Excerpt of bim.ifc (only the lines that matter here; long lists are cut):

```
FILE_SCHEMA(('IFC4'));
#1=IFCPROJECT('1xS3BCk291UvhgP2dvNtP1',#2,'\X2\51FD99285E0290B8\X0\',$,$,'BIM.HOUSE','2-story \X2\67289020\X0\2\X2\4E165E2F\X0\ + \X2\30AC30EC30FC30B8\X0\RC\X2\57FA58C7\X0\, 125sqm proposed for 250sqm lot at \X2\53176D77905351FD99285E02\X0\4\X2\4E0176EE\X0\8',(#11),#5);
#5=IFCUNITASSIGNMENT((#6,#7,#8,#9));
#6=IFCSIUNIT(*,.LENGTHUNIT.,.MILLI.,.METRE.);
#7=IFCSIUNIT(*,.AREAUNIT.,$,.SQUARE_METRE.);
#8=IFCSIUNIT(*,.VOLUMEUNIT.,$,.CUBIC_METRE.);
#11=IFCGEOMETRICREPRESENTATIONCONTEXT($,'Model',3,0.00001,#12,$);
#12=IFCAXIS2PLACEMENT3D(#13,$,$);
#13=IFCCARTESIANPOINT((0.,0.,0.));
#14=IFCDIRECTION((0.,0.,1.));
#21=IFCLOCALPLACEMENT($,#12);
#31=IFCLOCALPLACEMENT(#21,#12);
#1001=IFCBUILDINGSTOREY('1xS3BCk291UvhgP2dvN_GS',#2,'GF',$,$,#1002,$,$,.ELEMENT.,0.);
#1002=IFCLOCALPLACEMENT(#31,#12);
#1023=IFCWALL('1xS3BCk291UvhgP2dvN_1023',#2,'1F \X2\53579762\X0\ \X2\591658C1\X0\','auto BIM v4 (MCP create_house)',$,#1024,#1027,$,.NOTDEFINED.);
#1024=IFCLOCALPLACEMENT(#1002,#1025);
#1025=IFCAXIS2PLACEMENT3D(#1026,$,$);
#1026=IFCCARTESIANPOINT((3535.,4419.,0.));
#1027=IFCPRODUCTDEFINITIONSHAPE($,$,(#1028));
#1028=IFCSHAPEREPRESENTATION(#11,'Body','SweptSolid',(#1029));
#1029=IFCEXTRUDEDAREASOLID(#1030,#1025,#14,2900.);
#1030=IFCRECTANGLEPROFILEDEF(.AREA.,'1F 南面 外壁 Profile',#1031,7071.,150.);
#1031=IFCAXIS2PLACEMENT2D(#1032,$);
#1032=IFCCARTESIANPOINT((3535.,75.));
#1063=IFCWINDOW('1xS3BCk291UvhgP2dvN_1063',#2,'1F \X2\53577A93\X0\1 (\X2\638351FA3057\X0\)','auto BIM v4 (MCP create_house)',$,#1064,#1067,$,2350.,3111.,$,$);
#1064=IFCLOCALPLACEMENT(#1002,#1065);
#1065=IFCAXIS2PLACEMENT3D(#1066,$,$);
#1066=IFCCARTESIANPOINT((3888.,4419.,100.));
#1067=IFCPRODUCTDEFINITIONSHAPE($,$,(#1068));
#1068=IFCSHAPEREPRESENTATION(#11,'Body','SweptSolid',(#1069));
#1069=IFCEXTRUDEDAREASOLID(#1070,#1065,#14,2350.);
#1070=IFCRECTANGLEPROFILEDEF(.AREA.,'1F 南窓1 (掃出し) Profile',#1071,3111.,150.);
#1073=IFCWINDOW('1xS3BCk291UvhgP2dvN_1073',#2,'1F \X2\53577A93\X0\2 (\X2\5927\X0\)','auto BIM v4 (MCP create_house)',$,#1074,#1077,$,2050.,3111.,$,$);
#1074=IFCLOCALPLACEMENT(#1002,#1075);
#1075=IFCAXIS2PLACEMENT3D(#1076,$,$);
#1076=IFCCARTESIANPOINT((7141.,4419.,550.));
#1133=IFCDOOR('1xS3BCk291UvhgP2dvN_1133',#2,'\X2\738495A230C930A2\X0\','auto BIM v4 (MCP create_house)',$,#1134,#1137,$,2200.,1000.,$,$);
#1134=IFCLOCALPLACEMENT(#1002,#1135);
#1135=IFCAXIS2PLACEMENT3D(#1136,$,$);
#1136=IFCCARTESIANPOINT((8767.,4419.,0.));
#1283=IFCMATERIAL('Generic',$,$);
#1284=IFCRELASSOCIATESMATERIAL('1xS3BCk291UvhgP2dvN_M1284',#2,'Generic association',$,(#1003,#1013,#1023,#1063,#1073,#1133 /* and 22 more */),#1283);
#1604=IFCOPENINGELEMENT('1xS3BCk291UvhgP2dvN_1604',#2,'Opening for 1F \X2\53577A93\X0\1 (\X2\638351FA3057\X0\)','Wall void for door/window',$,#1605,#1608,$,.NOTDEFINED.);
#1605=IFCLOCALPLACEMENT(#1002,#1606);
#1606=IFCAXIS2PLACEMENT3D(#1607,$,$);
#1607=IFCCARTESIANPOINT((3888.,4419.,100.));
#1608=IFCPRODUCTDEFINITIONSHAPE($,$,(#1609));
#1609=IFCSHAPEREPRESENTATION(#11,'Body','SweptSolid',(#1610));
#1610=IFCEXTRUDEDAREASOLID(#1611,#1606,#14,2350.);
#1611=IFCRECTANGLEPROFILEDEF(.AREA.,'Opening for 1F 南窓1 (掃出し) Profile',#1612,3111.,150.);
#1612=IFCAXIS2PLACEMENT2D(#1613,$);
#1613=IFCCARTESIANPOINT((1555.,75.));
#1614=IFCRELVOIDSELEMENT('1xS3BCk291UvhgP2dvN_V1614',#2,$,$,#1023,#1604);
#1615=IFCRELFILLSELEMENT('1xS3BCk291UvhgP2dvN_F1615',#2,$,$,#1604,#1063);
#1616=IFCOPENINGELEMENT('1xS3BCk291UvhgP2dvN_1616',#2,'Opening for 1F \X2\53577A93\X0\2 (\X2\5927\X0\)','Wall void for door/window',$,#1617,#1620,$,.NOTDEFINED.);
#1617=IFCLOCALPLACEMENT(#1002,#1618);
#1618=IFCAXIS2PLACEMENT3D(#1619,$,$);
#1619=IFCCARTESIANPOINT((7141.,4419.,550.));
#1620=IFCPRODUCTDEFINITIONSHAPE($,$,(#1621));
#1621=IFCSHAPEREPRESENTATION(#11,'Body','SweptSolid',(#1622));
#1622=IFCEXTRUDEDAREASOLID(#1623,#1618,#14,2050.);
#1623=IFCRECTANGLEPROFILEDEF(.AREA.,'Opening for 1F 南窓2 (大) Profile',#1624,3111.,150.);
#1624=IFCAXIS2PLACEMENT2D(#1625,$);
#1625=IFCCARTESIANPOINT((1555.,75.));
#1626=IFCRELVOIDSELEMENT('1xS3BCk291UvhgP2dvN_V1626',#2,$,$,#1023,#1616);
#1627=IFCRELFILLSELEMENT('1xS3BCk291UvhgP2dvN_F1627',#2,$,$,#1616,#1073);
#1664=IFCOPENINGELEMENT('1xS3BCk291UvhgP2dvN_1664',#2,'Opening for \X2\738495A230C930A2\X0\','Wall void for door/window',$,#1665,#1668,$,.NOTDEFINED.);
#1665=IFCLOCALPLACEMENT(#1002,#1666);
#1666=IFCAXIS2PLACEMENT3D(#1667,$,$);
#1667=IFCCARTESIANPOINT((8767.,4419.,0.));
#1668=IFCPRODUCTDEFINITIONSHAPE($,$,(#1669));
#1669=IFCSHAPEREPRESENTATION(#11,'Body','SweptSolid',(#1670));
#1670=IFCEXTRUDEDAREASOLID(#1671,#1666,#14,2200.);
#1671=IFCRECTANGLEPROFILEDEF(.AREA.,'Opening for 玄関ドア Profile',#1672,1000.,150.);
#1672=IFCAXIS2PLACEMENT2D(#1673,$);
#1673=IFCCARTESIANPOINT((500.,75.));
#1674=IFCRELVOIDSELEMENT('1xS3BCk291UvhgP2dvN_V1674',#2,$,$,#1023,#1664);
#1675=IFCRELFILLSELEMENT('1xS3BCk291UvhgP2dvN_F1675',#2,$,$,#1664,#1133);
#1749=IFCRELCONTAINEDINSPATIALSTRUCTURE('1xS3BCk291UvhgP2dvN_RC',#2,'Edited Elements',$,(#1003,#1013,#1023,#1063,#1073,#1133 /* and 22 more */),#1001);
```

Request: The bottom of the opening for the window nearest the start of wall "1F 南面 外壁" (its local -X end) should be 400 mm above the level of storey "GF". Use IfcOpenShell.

```python
import numpy as np
import ifcopenshell
import ifcopenshell.api.geometry
import ifcopenshell.geom
import ifcopenshell.util.element
import ifcopenshell.util.placement
import ifcopenshell.util.shape
import ifcopenshell.util.unit

model = ifcopenshell.open("bim.ifc")
unit_scale = ifcopenshell.util.unit.calculate_unit_scale(model)

window = model.by_guid("1xS3BCk291UvhgP2dvN_1063")
opening = window.FillsVoids[0].RelatingOpeningElement
storey = ifcopenshell.util.element.get_container(window, ifc_class="IfcBuildingStorey")
level = ifcopenshell.util.placement.get_local_placement(storey.ObjectPlacement)[2, 3]

# The opening's origin need not be at the sill, so measure its lowest point.
shape = ifcopenshell.geom.create_shape(ifcopenshell.geom.settings(), opening)
bottom = ifcopenshell.util.shape.get_shape_bottom_elevation(shape, shape.geometry) / unit_scale
dz = level + 400.0 - bottom

shift = np.array([0.0, 0.0, dz])
# The window is not placed relative to its opening, so move both.
for product in (opening, window):
    matrix = ifcopenshell.util.placement.get_local_placement(product.ObjectPlacement)
    matrix[:3, 3] += shift
    ifcopenshell.api.geometry.edit_object_placement(model, product=product, matrix=matrix, is_si=False)

print(f"moved by {dz * unit_scale:+.3f} m")

model.write("bim_rev.ifc")
```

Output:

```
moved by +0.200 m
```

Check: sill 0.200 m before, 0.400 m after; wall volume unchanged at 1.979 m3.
